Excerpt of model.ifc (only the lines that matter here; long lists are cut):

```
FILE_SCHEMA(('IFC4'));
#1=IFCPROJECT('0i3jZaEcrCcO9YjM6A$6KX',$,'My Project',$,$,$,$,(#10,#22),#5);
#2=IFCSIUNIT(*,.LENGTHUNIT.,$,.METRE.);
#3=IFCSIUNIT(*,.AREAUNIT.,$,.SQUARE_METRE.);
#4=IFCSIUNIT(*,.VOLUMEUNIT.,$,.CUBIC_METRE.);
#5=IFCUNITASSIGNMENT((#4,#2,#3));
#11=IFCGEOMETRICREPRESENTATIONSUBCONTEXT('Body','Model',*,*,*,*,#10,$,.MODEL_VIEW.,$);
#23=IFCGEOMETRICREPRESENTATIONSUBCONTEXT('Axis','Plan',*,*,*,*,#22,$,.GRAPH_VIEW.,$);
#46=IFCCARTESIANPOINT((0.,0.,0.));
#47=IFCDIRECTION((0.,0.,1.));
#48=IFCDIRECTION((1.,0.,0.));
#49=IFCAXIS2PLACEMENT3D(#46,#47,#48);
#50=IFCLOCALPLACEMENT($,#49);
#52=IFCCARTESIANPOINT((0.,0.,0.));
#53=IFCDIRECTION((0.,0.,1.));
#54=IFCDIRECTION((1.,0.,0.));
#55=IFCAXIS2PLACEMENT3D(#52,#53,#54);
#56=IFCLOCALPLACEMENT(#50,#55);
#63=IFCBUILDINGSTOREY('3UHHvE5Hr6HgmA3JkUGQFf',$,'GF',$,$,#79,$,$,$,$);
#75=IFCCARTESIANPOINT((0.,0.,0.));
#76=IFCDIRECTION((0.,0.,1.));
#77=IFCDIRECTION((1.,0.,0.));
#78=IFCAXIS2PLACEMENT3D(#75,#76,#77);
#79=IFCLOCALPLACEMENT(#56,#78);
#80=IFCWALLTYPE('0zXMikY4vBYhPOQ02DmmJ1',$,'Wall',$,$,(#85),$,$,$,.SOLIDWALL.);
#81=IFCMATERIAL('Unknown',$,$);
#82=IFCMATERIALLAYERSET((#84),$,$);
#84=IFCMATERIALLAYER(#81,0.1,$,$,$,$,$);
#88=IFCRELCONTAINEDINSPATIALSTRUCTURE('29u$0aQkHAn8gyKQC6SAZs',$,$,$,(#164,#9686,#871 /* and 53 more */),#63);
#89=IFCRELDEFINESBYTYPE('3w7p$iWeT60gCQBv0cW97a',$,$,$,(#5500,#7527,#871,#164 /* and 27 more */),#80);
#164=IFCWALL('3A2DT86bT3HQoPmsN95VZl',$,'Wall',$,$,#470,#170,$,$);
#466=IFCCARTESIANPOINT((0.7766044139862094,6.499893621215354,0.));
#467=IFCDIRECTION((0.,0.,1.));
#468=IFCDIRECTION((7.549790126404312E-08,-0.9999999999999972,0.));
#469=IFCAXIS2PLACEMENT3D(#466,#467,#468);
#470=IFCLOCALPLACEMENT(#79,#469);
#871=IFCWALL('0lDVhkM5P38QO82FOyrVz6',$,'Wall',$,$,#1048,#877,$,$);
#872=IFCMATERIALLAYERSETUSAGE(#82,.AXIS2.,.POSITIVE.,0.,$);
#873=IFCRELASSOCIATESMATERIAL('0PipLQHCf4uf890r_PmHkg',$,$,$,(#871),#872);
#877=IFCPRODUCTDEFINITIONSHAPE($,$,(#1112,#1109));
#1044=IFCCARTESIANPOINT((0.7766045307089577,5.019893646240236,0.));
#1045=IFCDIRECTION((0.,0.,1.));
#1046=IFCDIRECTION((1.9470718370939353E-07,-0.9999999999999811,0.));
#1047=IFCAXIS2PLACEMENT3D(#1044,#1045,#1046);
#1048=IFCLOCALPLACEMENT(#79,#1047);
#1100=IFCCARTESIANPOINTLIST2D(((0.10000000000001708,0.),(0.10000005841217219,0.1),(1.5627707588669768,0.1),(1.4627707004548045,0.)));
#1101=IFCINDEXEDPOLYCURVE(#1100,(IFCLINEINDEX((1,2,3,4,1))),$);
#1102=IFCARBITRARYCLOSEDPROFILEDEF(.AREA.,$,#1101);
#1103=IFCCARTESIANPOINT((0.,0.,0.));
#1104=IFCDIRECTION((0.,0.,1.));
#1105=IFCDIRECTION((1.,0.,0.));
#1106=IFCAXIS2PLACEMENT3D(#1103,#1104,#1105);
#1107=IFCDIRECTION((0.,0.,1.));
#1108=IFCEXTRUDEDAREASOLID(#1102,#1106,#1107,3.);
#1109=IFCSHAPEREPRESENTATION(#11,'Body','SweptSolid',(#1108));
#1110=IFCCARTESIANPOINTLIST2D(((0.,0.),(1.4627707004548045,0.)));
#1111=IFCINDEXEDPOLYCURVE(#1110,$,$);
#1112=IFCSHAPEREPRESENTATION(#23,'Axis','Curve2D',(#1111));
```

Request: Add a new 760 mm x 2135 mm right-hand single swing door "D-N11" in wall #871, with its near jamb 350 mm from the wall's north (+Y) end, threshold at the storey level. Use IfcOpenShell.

```python
import numpy as np
import ifcopenshell
import ifcopenshell.api.feature
import ifcopenshell.api.geometry
import ifcopenshell.api.root
import ifcopenshell.api.spatial
import ifcopenshell.geom
import ifcopenshell.util.element
import ifcopenshell.util.placement
import ifcopenshell.util.representation
import ifcopenshell.util.shape
import ifcopenshell.util.unit

model = ifcopenshell.open("model.ifc")
unit_scale = ifcopenshell.util.unit.calculate_unit_scale(model)
settings = ifcopenshell.geom.settings()


def volume(element):
    """Net volume in cubic metres, openings subtracted."""
    shape = ifcopenshell.geom.create_shape(settings, element)
    return ifcopenshell.util.shape.get_volume(shape.geometry)


wall = model.by_guid("0lDVhkM5P38QO82FOyrVz6")
storey = ifcopenshell.util.element.get_container(wall, ifc_class="IfcBuildingStorey")
context = ifcopenshell.util.representation.get_context(model, "Model", "Body", "MODEL_VIEW")
before = volume(wall)

width, height, from_end, sill = 0.76, 2.135, 0.35, 0.0  # metres

# The wall runs along its own X axis, and the end named is its -X end.
wall_shape = ifcopenshell.geom.create_shape(settings, wall)
x, y, z = ifcopenshell.util.shape.get_vertices(wall_shape.geometry).T
start = x.min() + from_end
face, thickness = float(y.min()), float(y.max() - y.min())
wall_matrix = ifcopenshell.util.placement.get_local_placement(wall.ObjectPlacement)
level = ifcopenshell.util.placement.get_local_placement(storey.ObjectPlacement)[2, 3]


def in_wall(x, y):
    """Placement at x, y metres in the wall's axes, at sill height."""
    matrix = wall_matrix.copy()
    matrix[:, 3] = wall_matrix @ np.array([x / unit_scale, y / unit_scale, 0.0, 1.0])
    matrix[2, 3] = level + sill / unit_scale
    return matrix


# Opening: a box that overshoots both wall faces by 50 mm.
opening = ifcopenshell.api.root.create_entity(model, ifc_class="IfcOpeningElement", predefined_type="OPENING")
box = ifcopenshell.api.geometry.add_wall_representation(
    model, context=context, length=width, height=height, thickness=thickness + 0.1
)
ifcopenshell.api.geometry.assign_representation(model, product=opening, representation=box)
ifcopenshell.api.geometry.edit_object_placement(model, product=opening, matrix=in_wall(start, face - 0.05), is_si=False)
ifcopenshell.api.feature.add_feature(model, feature=opening, element=wall)

door = ifcopenshell.api.root.create_entity(model, ifc_class="IfcDoor", name="D-N11", predefined_type="DOOR")
door.OverallWidth, door.OverallHeight = width / unit_scale, height / unit_scale
door.OperationType = "SINGLE_SWING_RIGHT"
body = ifcopenshell.api.geometry.add_door_representation(
    model,
    context=context,
    overall_width=door.OverallWidth,
    overall_height=door.OverallHeight,
    operation_type="SINGLE_SWING_RIGHT",
    lining_properties={"LiningDepth": thickness / unit_scale, "ThresholdDepth": thickness / unit_scale},
)
ifcopenshell.api.geometry.assign_representation(model, product=door, representation=body)
ifcopenshell.api.spatial.assign_container(model, products=[door], relating_structure=storey)
ifcopenshell.api.feature.add_filling(model, opening=opening, element=door)

# The lining spans the wall, so the door starts at the wall face.
ifcopenshell.api.geometry.edit_object_placement(model, product=door, matrix=in_wall(start, face), is_si=False)

after = volume(wall)

print(f"wall volume {before:.3f} -> {after:.3f} m3")

model.write("model_edited.ifc")
```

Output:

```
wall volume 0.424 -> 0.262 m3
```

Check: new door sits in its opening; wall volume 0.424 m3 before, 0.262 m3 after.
